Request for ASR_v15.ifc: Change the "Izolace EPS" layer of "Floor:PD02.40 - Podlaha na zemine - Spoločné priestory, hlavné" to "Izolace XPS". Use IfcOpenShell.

First a look at what the model holds.

```python
import ifcopenshell
import ifcopenshell.util.element

model = ifcopenshell.open("ASR_v15.ifc")
print(model.schema)
for layer_set in model.by_type("IfcMaterialLayerSet"):
    if layer_set.LayerSetName == "Floor:PD02.40 - Podlaha na zemine - Spoločné priestory, hlavné":
        for layer in layer_set.MaterialLayers:
            print(layer.id(), layer.Material and layer.Material.Name, layer.LayerThickness, sep=" | ")
        print(len(ifcopenshell.util.element.get_elements_by_material(model, layer_set)), "elements and types use it")
print(sorted(m.Name for m in model.by_type("IfcMaterial") if m.Name)[:60])
```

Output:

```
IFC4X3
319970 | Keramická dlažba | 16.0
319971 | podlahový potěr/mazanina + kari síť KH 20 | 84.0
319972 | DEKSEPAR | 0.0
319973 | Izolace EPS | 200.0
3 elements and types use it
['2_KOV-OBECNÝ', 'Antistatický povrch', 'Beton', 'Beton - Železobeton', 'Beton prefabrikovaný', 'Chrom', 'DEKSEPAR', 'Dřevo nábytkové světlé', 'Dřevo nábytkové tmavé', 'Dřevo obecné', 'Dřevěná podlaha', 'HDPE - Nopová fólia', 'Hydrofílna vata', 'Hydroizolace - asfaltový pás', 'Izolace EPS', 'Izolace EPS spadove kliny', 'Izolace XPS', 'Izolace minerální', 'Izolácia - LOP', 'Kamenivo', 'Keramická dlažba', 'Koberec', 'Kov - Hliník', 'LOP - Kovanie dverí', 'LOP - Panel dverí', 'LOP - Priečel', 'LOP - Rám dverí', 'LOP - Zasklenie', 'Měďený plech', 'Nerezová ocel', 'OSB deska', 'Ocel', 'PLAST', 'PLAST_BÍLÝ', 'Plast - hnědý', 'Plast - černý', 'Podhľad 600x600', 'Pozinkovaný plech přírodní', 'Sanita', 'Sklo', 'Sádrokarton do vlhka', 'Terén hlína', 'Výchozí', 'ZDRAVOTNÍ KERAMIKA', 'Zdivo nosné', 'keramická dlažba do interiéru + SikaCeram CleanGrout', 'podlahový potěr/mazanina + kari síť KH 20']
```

```python
import ifcopenshell
import ifcopenshell.api.material

model = ifcopenshell.open("ASR_v15.ifc")

layer_set = next(s for s in model.by_type("IfcMaterialLayerSet") if s.LayerSetName == "Floor:PD02.40 - Podlaha na zemine - Spoločné priestory, hlavné")
layer = next(l for l in layer_set.MaterialLayers if l.Material and l.Material.Name == "Izolace EPS")
material = next(m for m in model.by_type("IfcMaterial") if m.Name == "Izolace XPS")

# Point this one layer at the other material; renaming the old one would change it everywhere.
ifcopenshell.api.material.edit_layer(model, layer=layer, attributes={"Name": material.Name}, material=material)

print([l.Material.Name if l.Material else None for l in layer_set.MaterialLayers])

model.write("ASR_v15_edited.ifc")
```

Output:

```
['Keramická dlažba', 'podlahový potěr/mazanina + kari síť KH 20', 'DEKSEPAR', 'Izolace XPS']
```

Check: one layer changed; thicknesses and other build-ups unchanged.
